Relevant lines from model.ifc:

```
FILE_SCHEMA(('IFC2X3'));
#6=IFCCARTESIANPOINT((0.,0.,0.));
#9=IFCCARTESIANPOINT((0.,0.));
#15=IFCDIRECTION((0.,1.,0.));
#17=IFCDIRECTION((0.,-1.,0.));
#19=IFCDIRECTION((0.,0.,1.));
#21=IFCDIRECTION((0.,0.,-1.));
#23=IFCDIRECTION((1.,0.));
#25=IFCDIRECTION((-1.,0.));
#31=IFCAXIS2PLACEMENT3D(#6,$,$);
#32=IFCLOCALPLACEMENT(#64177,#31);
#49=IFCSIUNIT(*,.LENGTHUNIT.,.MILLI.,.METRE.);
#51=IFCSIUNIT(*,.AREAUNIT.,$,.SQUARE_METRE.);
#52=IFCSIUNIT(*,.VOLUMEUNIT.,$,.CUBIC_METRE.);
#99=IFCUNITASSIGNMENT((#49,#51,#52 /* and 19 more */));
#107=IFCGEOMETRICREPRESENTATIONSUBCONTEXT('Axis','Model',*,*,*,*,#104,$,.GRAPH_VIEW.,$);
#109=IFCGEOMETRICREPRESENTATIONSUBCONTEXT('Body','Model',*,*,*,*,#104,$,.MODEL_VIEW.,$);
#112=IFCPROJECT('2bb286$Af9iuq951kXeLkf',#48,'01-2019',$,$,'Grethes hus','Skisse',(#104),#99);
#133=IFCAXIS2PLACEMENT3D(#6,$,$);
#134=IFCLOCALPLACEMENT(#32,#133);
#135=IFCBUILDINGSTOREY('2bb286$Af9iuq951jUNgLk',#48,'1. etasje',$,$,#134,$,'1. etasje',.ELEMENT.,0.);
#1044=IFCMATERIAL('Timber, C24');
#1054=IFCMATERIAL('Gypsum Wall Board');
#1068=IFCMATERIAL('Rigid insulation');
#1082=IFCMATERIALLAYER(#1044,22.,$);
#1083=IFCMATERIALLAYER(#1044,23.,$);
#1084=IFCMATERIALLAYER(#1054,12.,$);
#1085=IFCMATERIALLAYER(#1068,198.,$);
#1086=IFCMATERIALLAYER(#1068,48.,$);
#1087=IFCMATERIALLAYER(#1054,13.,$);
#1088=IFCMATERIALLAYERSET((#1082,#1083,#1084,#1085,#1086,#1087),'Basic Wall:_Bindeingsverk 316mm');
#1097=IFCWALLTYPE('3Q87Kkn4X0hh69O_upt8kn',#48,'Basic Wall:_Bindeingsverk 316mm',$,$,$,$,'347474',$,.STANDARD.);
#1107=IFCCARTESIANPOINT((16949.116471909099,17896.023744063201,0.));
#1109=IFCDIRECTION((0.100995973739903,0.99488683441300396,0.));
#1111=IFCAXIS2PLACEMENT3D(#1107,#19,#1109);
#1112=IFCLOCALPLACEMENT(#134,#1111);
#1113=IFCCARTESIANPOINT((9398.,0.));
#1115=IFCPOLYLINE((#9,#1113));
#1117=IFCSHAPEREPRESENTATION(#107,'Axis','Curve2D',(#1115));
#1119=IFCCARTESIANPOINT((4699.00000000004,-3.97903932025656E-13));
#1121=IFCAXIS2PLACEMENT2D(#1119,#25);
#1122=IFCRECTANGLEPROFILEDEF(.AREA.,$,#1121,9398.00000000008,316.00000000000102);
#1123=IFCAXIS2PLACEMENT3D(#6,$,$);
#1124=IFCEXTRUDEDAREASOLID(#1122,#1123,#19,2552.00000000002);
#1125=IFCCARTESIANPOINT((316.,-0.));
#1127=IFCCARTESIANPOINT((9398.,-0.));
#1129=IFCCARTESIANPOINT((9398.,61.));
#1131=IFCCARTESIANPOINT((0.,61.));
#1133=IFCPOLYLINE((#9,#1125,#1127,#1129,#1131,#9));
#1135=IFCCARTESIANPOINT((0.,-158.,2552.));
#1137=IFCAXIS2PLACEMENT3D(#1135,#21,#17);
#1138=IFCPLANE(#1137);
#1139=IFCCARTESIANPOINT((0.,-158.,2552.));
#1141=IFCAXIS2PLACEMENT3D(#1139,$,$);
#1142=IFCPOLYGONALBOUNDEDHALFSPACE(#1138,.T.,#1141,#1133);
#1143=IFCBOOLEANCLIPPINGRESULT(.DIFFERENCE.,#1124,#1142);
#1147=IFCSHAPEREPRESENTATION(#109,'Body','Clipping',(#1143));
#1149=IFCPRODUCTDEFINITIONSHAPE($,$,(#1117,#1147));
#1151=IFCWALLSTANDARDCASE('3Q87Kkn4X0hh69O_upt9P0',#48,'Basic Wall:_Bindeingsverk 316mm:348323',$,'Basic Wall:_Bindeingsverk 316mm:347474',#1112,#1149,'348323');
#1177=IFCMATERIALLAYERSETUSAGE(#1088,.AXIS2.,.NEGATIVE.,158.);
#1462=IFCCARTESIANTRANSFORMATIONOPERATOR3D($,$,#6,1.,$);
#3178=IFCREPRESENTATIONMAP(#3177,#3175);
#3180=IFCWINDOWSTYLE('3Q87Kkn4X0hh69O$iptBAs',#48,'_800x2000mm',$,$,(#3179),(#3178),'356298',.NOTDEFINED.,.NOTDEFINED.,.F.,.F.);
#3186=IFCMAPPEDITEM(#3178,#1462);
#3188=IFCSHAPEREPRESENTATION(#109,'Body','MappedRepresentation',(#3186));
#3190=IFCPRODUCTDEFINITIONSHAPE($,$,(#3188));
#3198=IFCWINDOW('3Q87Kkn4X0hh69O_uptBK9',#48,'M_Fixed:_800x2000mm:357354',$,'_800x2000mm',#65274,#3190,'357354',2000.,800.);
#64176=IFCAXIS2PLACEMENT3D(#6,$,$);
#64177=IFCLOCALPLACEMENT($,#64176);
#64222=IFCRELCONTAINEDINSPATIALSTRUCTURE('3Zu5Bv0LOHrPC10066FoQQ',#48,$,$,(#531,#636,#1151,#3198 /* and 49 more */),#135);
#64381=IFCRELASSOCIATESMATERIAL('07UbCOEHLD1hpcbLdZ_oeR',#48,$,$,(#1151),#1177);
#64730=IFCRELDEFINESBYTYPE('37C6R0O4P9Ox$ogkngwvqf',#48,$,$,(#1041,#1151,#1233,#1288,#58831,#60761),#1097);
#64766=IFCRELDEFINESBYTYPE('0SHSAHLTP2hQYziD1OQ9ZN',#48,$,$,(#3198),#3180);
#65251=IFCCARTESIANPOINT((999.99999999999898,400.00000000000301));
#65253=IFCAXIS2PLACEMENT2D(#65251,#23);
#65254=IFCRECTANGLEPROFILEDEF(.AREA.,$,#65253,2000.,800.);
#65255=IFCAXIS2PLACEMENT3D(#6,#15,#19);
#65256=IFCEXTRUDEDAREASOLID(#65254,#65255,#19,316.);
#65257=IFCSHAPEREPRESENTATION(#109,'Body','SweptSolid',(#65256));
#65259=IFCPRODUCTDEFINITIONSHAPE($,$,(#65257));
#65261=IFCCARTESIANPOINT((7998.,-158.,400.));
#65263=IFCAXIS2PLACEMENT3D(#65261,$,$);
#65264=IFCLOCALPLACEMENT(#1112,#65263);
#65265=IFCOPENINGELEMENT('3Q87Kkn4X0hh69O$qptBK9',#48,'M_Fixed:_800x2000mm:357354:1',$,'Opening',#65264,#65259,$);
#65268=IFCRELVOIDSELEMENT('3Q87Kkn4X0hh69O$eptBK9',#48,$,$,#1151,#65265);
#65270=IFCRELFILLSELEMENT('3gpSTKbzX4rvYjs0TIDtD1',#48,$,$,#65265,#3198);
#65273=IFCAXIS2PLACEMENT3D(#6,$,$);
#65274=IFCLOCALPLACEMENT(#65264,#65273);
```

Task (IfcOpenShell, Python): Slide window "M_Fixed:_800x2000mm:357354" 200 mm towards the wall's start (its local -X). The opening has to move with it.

```python
import ifcopenshell
import ifcopenshell.api.geometry
import ifcopenshell.util.placement
import ifcopenshell.util.unit

model = ifcopenshell.open("model.ifc")
unit_scale = ifcopenshell.util.unit.calculate_unit_scale(model)

window = model.by_id(3198)
opening = window.FillsVoids[0].RelatingOpeningElement
wall = opening.VoidsElements[0].RelatingBuildingElement

wall_matrix = ifcopenshell.util.placement.get_local_placement(wall.ObjectPlacement)
shift = wall_matrix[:3, 0] * -0.2 / unit_scale
before = ifcopenshell.util.placement.get_local_placement(window.ObjectPlacement)[:3, 3].copy()

# The window is placed relative to its opening, so it follows when the opening moves.
matrix = ifcopenshell.util.placement.get_local_placement(opening.ObjectPlacement)
matrix[:3, 3] += shift
ifcopenshell.api.geometry.edit_object_placement(
    model, product=opening, matrix=matrix, is_si=False, should_transform_children=True
)

after = ifcopenshell.util.placement.get_local_placement(window.ObjectPlacement)[:3, 3]
print("window moved by", (after - before).round(3) + 0.0)

model.write("model_edited.ifc")
```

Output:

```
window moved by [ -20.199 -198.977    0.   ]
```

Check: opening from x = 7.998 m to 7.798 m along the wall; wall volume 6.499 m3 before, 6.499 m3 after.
